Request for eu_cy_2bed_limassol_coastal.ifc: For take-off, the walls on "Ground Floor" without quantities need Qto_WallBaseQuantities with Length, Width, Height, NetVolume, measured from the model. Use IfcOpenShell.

First a look at what the model holds.

```python
import ifcopenshell
import ifcopenshell.util.element
import ifcopenshell.util.unit

model = ifcopenshell.open("eu_cy_2bed_limassol_coastal.ifc")
print(model.schema)
for unit_type in ("LENGTHUNIT", "AREAUNIT", "VOLUMEUNIT"):
    print(unit_type, ifcopenshell.util.unit.calculate_unit_scale(model, unit_type))
storey = next(s for s in model.by_type("IfcBuildingStorey") if s.Name == "Ground Floor")
walls = [e for e in ifcopenshell.util.element.get_decomposition(storey) if e.is_a("IfcWall")]
for e in sorted(walls, key=lambda e: e.id()):
    print(e.id(), e.is_a(), e.Name, list(ifcopenshell.util.element.get_psets(e, qtos_only=True)), sep=" | ")
```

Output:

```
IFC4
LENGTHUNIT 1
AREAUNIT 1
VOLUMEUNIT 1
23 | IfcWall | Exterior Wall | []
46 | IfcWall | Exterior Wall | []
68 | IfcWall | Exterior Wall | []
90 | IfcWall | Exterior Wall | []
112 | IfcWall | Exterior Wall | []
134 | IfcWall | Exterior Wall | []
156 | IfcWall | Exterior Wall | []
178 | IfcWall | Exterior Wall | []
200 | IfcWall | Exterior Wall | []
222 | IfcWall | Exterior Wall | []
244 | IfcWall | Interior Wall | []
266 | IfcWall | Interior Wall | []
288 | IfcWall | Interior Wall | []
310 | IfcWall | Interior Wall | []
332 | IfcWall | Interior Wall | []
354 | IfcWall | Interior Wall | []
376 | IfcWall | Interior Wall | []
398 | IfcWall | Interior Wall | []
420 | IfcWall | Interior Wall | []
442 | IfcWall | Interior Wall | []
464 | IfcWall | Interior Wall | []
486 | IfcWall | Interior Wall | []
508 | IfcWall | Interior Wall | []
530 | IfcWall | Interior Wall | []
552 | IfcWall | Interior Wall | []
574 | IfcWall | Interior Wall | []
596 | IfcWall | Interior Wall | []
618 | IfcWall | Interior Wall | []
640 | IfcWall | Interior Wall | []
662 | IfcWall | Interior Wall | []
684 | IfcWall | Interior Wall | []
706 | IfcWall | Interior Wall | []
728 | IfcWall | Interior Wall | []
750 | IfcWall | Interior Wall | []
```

```python
import ifcopenshell
import ifcopenshell.api.pset
import ifcopenshell.geom
import ifcopenshell.util.element
import ifcopenshell.util.shape
import ifcopenshell.util.unit

model = ifcopenshell.open("eu_cy_2bed_limassol_coastal.ifc")
unit_scale = ifcopenshell.util.unit.calculate_unit_scale(model)
volume_scale = ifcopenshell.util.unit.calculate_unit_scale(model, "VOLUMEUNIT")
settings = ifcopenshell.geom.settings()

storey = next(s for s in model.by_type("IfcBuildingStorey") if s.Name == "Ground Floor")
walls = [e for e in ifcopenshell.util.element.get_decomposition(storey) if e.is_a("IfcWall")]

for e in sorted(walls, key=lambda e: e.id()):
    if ifcopenshell.util.element.get_psets(e, qtos_only=True, should_inherit=False):
        continue
    # Geometry comes back in metres, in the element's own axes.
    shape = ifcopenshell.geom.create_shape(settings, e)
    values = {
        "Length": ifcopenshell.util.shape.get_x(shape.geometry) / unit_scale,
        "Width": ifcopenshell.util.shape.get_y(shape.geometry) / unit_scale,
        "Height": ifcopenshell.util.shape.get_z(shape.geometry) / unit_scale,
        "NetVolume": ifcopenshell.util.shape.get_volume(shape.geometry) / volume_scale,
    }
    qto = ifcopenshell.api.pset.add_qto(model, product=e, name="Qto_WallBaseQuantities")
    ifcopenshell.api.pset.edit_qto(model, qto=qto, properties=values)
    print(e.id(), {k: round(v, 3) for k, v in values.items()})

model.write("eu_cy_2bed_limassol_coastal_v2.ifc")
```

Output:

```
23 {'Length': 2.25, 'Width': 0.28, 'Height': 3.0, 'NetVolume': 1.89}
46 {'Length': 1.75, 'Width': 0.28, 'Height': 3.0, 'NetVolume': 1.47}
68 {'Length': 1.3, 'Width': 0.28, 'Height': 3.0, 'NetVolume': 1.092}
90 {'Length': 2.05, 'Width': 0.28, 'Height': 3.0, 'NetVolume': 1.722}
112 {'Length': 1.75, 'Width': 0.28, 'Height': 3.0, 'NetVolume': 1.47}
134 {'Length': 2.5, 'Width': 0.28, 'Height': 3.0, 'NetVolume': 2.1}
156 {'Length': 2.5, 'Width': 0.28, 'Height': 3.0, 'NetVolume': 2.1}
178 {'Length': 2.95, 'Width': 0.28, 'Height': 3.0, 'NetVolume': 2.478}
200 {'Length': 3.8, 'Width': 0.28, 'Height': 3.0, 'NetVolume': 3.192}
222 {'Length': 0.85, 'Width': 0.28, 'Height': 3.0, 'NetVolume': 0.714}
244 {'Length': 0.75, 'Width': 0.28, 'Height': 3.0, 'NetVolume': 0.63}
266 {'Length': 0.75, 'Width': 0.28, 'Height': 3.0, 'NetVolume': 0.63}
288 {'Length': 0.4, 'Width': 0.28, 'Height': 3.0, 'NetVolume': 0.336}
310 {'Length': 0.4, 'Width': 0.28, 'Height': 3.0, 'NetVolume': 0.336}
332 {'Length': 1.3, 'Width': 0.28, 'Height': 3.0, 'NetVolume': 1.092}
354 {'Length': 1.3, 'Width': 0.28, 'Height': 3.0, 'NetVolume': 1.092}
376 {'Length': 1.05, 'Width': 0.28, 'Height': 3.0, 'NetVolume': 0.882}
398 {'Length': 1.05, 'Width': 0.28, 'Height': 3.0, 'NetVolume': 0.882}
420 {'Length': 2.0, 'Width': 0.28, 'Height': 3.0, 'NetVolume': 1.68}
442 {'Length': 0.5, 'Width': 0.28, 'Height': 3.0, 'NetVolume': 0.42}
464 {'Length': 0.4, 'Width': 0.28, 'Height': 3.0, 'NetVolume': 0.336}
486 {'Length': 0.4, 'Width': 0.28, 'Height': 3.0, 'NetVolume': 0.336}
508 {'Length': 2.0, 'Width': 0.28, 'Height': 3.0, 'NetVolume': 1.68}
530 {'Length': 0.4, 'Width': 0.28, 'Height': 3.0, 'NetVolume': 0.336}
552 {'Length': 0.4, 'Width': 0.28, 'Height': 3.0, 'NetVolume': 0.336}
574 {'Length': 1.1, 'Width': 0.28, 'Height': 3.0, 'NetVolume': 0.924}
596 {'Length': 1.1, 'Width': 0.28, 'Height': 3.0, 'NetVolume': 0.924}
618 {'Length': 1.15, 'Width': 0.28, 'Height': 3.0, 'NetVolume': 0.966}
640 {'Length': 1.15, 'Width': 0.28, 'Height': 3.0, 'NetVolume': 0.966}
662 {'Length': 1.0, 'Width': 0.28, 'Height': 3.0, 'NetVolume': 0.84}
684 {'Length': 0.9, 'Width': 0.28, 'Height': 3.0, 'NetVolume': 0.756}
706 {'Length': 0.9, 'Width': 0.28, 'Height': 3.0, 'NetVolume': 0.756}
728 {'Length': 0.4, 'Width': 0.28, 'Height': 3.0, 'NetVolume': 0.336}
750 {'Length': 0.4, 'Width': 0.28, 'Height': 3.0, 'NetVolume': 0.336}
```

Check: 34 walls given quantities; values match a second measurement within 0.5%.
